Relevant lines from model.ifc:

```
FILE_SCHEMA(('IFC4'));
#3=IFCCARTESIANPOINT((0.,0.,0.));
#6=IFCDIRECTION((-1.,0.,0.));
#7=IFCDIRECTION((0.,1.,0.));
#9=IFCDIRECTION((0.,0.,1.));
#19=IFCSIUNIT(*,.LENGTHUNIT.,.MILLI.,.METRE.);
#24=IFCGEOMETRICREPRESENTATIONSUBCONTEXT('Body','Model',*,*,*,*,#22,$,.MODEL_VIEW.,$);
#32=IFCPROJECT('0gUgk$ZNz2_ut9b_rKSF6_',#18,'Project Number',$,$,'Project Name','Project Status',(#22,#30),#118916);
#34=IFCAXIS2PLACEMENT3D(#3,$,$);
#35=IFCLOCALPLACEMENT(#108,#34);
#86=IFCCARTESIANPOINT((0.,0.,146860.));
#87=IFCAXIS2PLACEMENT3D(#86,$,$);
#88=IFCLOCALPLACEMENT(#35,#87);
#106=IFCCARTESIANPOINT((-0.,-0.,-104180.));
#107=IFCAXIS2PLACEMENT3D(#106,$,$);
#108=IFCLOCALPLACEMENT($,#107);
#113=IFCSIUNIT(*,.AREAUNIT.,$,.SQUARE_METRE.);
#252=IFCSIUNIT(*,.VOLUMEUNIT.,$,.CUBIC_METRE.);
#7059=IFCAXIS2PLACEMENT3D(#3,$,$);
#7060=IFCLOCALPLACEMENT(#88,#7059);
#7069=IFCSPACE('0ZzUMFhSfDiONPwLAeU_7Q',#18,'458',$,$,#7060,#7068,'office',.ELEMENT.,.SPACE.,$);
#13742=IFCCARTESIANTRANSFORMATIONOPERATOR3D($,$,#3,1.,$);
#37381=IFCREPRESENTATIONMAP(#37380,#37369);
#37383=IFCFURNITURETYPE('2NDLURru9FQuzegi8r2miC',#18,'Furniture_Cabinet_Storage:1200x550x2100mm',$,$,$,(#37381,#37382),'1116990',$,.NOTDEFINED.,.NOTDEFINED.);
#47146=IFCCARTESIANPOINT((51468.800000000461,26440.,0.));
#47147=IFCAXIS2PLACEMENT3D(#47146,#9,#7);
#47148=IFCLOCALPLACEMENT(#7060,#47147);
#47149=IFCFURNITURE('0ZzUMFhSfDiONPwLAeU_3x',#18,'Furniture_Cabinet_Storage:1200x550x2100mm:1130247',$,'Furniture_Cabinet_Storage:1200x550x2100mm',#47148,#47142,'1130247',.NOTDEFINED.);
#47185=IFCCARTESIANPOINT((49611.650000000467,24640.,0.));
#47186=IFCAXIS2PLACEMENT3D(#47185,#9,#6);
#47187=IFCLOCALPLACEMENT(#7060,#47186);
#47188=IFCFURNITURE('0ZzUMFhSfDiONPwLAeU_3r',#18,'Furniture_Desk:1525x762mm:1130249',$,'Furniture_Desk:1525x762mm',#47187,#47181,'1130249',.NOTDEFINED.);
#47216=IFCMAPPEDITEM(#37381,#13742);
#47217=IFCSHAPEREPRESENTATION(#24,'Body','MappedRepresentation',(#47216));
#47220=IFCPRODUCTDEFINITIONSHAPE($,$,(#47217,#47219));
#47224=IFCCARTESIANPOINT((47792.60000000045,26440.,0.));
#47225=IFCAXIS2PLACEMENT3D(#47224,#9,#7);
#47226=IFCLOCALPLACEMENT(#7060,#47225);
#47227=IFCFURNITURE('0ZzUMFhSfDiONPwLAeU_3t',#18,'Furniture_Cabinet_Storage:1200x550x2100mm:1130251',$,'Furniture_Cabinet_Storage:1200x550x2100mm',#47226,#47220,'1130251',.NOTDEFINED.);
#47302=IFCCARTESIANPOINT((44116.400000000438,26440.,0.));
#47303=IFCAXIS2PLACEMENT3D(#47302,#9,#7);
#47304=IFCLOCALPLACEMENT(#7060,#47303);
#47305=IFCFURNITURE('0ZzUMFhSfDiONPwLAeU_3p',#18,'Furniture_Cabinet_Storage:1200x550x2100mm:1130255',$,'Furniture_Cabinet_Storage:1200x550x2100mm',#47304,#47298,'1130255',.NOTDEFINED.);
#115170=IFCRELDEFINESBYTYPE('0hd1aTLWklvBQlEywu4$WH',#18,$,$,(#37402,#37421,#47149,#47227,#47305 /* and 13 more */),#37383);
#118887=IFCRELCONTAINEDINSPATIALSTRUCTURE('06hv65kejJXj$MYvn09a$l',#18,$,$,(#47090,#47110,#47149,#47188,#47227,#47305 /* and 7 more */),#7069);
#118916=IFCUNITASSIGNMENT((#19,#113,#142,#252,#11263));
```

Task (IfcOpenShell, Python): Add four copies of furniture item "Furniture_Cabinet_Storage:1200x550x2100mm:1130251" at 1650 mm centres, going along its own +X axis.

```python
import ifcopenshell
import ifcopenshell.api.geometry
import ifcopenshell.api.root
import ifcopenshell.util.element
import ifcopenshell.util.placement

model = ifcopenshell.open("model.ifc")


def reuse_history(source, copy):
    """copy_class also copies each property set's owner history, people and application; keep the originals."""
    for rel in copy.IsDefinedBy:
        if rel.is_a("IfcRelDefinesByProperties") and (history := rel.RelatingPropertyDefinition.OwnerHistory):
            rel.RelatingPropertyDefinition.OwnerHistory = source.OwnerHistory
            ifcopenshell.util.element.remove_deep2(model, history)


source = model.by_id(47227)
base = ifcopenshell.util.placement.get_local_placement(source.ObjectPlacement)
step = base[:3, 0] * 1650.0

for i in range(1, 5):
    copy = ifcopenshell.api.root.copy_class(model, product=source)
    copy.Representation = ifcopenshell.util.element.copy_deep(
        model, source.Representation, exclude=["IfcGeometricRepresentationContext", "IfcRepresentationMap"]
    )
    copy.Name = "Furniture_Cabinet_Storage:1200x550x2100mm"
    copy.Tag = None
    reuse_history(source, copy)
    matrix = base.copy()
    matrix[:3, 3] += i * step
    print("added at", matrix[:3, 3].round(3) + 0.0)
    ifcopenshell.api.geometry.edit_object_placement(model, product=copy, matrix=matrix, is_si=False)

model.write("model_v2.ifc")
```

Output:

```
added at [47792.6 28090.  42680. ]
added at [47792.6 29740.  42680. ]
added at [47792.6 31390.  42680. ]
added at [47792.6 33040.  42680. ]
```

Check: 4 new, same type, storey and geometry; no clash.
